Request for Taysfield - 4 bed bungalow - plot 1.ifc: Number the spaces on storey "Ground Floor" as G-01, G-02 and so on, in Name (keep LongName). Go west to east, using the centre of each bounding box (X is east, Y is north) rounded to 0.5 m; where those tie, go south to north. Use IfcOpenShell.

First a look at what the model holds.

```python
import ifcopenshell
import ifcopenshell.util.element
import ifcopenshell.util.placement

model = ifcopenshell.open("Taysfield - 4 bed bungalow - plot 1.ifc")
print(model.schema)
storey = next(s for s in model.by_type("IfcBuildingStorey") if s.Name == "Ground Floor")
spaces = [e for e in ifcopenshell.util.element.get_decomposition(storey) if e.is_a("IfcSpace")]
for e in sorted(spaces, key=lambda e: e.id()):
    origin = ifcopenshell.util.placement.get_local_placement(e.ObjectPlacement)[:3, 3]
    print(e.id(), e.Name, e.LongName, origin.round(2) + 0.0, sep=" | ")
```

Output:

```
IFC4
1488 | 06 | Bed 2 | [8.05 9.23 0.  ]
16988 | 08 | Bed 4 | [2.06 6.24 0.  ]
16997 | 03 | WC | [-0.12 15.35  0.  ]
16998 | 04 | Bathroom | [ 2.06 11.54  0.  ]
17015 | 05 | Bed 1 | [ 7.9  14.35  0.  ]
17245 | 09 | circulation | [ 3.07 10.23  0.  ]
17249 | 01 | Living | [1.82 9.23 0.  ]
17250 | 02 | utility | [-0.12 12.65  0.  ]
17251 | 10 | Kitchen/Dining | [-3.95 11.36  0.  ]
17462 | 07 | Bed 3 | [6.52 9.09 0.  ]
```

```python
import ifcopenshell
import ifcopenshell.geom
import ifcopenshell.util.element
import ifcopenshell.util.shape

model = ifcopenshell.open("Taysfield - 4 bed bungalow - plot 1.ifc")
settings = ifcopenshell.geom.settings()
settings.set("use-world-coords", True)


def centre(element):
    shape = ifcopenshell.geom.create_shape(settings, element)
    return ifcopenshell.util.shape.get_bbox_centroid(shape.geometry)


storey = next(s for s in model.by_type("IfcBuildingStorey") if s.Name == "Ground Floor")
spaces = [e for e in ifcopenshell.util.element.get_decomposition(storey) if e.is_a("IfcSpace")]

# Insertion points can sit at a corner or the storey origin, so sort by the geometry (in metres).
centres = {e: centre(e) for e in spaces}
spaces.sort(key=lambda e: (round(centres[e][0] / 0.5), centres[e][1]))

for i, e in enumerate(spaces, start=1):
    number = f"G-{i:02d}"
    e.Name = number
    print(e.id(), number)

model.write("Taysfield - 4 bed bungalow - plot 1_updated.ifc")
```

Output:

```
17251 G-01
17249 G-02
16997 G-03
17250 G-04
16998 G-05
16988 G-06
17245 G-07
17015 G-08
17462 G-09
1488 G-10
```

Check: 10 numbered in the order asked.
